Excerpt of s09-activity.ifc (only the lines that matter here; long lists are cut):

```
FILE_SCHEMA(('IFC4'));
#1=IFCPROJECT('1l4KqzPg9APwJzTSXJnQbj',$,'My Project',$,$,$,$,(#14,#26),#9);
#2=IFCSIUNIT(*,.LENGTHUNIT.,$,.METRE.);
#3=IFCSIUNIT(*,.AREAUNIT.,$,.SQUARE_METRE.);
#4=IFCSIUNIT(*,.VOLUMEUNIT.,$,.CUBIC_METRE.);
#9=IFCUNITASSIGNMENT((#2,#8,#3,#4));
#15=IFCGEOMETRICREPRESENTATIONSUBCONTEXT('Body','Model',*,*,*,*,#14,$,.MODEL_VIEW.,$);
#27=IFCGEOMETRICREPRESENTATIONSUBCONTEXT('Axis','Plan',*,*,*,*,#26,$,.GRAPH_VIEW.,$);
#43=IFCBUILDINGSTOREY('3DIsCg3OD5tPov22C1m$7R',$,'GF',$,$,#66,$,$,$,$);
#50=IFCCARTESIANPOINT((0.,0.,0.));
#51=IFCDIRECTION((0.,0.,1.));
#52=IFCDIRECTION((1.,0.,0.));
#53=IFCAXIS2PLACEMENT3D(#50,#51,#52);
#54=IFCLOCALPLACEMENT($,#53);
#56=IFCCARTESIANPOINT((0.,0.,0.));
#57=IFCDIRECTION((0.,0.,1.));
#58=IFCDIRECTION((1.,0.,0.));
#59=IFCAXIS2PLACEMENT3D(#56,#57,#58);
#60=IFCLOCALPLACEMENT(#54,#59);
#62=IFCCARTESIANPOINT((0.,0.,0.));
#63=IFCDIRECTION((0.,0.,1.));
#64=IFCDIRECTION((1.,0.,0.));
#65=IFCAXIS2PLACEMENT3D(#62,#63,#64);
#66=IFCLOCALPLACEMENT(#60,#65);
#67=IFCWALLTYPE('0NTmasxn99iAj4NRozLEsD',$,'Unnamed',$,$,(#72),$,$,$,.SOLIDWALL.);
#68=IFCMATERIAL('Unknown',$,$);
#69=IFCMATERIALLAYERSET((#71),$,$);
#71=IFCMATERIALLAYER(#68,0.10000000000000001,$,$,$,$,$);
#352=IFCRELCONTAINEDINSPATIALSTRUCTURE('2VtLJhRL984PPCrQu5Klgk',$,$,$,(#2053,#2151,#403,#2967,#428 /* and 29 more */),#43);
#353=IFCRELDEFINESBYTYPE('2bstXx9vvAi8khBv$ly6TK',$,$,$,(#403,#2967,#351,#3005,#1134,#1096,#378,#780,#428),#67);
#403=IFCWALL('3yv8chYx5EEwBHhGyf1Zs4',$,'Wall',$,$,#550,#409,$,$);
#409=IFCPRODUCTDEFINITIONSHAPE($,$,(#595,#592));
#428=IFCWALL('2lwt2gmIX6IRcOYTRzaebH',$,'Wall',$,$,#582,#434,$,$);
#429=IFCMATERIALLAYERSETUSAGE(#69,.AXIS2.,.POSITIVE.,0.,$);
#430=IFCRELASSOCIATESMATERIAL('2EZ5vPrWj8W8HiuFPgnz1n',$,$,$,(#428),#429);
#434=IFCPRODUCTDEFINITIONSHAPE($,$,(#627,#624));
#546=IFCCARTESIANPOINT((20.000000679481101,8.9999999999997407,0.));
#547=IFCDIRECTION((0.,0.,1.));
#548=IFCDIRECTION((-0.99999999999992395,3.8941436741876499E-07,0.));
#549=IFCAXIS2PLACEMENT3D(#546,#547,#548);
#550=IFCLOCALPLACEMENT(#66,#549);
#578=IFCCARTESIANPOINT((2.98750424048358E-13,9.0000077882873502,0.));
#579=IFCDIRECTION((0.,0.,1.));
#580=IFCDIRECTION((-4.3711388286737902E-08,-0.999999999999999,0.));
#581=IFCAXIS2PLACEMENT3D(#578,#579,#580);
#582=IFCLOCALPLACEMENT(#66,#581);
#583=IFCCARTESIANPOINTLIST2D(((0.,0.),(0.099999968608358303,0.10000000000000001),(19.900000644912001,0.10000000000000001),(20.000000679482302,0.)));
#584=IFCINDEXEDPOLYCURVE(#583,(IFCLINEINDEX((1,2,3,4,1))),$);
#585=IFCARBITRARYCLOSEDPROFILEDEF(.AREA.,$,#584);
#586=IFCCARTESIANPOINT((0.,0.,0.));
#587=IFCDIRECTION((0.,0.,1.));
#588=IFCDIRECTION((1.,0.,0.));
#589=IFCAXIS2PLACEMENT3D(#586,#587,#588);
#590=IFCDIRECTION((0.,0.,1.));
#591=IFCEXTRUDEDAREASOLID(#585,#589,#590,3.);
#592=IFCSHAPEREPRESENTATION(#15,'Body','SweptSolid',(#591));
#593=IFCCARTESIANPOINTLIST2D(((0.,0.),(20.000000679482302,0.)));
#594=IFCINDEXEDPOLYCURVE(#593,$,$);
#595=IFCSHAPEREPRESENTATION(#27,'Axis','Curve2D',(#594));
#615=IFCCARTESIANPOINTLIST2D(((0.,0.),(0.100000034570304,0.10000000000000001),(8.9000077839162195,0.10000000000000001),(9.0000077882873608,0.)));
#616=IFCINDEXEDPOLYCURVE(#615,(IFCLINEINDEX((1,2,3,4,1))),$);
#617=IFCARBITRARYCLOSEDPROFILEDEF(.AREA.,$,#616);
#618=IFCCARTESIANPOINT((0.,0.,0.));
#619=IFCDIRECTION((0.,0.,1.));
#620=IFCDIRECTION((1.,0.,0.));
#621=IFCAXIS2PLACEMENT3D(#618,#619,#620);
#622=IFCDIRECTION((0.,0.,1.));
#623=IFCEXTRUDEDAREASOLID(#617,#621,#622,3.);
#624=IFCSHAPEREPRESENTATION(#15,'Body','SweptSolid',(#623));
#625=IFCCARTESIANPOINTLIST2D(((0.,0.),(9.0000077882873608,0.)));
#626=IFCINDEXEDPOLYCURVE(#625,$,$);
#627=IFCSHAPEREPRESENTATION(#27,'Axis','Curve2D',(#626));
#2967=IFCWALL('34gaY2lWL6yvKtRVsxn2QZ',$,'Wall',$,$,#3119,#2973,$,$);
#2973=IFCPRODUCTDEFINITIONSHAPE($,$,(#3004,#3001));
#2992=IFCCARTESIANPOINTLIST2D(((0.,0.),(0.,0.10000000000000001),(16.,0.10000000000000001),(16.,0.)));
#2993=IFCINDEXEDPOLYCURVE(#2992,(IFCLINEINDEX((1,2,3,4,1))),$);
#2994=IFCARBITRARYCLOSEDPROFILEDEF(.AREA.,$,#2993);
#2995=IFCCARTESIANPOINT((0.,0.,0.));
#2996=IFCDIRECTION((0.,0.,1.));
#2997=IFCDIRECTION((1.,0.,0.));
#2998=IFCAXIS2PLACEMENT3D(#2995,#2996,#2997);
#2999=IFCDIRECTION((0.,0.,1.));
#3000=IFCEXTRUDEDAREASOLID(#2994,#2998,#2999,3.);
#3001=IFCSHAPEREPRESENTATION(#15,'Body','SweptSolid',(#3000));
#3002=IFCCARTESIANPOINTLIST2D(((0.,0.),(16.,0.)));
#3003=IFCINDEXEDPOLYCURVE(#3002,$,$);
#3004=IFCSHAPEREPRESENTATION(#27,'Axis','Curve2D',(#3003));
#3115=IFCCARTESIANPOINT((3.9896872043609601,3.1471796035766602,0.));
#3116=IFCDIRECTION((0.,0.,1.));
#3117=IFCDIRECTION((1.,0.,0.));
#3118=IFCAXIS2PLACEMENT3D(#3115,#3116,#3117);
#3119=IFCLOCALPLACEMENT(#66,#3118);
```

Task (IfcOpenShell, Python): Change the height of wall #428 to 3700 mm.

```python
import ifcopenshell
import ifcopenshell.geom
import ifcopenshell.util.representation
import ifcopenshell.util.shape
import ifcopenshell.util.unit

model = ifcopenshell.open("s09-activity.ifc")
unit_scale = ifcopenshell.util.unit.calculate_unit_scale(model)
settings = ifcopenshell.geom.settings()


def volume(element):
    """Net volume in cubic metres, openings subtracted."""
    shape = ifcopenshell.geom.create_shape(settings, element)
    return ifcopenshell.util.shape.get_volume(shape.geometry)


wall = model.by_id(428)
before = volume(wall)

body = ifcopenshell.util.representation.get_representation(wall, "Model", "Body")
solid = body.Items[0]
old_height = solid.Depth
solid.Depth = 3.7 / unit_scale
after = volume(wall)

print(f"height {old_height:g} -> {solid.Depth:g}, volume {before:.3f} -> {after:.3f} m3")

model.write("s09-activity_v2.ifc")
```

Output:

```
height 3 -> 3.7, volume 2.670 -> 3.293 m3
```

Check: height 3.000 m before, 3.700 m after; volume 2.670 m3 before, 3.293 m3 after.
